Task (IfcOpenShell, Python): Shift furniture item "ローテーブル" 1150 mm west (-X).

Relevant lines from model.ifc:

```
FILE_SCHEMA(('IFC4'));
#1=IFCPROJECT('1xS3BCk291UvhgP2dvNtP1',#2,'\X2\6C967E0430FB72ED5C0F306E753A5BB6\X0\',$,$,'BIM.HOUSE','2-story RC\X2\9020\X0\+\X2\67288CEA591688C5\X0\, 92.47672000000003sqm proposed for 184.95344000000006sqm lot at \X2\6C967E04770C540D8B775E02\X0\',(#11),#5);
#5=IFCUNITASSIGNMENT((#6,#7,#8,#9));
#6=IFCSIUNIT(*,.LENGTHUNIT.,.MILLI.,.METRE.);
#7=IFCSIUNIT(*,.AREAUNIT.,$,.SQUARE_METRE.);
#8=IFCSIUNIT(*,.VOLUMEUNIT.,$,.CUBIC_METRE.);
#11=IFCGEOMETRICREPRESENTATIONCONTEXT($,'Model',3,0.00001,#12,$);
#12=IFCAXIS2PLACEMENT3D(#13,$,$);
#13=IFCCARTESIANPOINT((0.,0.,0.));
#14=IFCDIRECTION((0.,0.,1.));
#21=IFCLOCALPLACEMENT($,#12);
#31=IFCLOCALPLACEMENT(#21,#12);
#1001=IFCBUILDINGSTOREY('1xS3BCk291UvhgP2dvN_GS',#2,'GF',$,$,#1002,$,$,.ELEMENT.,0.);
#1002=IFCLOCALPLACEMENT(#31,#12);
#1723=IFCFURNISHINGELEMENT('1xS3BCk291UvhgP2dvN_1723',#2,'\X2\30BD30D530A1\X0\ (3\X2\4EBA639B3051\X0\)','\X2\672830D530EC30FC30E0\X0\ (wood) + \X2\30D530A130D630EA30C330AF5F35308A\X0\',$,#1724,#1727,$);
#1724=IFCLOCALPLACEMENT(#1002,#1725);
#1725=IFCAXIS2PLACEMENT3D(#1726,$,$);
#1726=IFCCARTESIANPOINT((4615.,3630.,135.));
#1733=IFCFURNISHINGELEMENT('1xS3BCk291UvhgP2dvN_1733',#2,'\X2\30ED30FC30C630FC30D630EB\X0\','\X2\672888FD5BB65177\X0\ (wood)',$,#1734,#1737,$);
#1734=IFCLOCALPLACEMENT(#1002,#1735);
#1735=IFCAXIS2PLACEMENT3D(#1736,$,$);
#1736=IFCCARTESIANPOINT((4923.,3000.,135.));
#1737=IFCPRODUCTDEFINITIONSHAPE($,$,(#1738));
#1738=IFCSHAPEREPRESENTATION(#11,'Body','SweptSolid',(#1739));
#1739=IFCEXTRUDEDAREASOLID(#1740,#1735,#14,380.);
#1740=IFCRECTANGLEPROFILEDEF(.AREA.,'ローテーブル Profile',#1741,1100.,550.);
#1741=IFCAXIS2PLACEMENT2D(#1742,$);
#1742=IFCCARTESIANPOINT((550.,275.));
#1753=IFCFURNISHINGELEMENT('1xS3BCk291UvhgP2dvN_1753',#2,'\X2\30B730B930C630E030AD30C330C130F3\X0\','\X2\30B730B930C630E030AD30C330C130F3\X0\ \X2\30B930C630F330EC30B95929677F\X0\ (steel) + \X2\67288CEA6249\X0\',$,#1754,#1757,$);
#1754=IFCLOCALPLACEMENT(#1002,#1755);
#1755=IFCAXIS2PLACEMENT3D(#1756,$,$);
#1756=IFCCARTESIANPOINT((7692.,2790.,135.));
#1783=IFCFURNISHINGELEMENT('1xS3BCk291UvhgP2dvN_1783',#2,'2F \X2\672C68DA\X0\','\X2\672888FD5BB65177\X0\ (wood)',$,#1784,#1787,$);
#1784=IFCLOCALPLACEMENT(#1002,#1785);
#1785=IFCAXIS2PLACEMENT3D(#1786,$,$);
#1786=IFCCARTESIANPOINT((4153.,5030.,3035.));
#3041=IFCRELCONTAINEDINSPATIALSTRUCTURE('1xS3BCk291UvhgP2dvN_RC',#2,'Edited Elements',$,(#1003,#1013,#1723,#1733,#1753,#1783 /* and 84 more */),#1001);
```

```python
import ifcopenshell
import ifcopenshell.api.geometry
import ifcopenshell.util.placement
import ifcopenshell.util.unit

model = ifcopenshell.open("model.ifc")
unit_scale = ifcopenshell.util.unit.calculate_unit_scale(model)

item = model.by_id(1733)
matrix = ifcopenshell.util.placement.get_local_placement(item.ObjectPlacement)
matrix[0, 3] -= 1.15 / unit_scale
ifcopenshell.api.geometry.edit_object_placement(model, product=item, matrix=matrix, is_si=False)

print(ifcopenshell.util.placement.get_local_placement(item.ObjectPlacement).round(3) + 0.0)

model.write("model_rev.ifc")
```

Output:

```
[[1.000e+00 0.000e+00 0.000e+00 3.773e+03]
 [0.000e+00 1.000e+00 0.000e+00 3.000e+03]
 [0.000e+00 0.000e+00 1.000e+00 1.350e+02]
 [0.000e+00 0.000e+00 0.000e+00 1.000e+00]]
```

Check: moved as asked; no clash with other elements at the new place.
